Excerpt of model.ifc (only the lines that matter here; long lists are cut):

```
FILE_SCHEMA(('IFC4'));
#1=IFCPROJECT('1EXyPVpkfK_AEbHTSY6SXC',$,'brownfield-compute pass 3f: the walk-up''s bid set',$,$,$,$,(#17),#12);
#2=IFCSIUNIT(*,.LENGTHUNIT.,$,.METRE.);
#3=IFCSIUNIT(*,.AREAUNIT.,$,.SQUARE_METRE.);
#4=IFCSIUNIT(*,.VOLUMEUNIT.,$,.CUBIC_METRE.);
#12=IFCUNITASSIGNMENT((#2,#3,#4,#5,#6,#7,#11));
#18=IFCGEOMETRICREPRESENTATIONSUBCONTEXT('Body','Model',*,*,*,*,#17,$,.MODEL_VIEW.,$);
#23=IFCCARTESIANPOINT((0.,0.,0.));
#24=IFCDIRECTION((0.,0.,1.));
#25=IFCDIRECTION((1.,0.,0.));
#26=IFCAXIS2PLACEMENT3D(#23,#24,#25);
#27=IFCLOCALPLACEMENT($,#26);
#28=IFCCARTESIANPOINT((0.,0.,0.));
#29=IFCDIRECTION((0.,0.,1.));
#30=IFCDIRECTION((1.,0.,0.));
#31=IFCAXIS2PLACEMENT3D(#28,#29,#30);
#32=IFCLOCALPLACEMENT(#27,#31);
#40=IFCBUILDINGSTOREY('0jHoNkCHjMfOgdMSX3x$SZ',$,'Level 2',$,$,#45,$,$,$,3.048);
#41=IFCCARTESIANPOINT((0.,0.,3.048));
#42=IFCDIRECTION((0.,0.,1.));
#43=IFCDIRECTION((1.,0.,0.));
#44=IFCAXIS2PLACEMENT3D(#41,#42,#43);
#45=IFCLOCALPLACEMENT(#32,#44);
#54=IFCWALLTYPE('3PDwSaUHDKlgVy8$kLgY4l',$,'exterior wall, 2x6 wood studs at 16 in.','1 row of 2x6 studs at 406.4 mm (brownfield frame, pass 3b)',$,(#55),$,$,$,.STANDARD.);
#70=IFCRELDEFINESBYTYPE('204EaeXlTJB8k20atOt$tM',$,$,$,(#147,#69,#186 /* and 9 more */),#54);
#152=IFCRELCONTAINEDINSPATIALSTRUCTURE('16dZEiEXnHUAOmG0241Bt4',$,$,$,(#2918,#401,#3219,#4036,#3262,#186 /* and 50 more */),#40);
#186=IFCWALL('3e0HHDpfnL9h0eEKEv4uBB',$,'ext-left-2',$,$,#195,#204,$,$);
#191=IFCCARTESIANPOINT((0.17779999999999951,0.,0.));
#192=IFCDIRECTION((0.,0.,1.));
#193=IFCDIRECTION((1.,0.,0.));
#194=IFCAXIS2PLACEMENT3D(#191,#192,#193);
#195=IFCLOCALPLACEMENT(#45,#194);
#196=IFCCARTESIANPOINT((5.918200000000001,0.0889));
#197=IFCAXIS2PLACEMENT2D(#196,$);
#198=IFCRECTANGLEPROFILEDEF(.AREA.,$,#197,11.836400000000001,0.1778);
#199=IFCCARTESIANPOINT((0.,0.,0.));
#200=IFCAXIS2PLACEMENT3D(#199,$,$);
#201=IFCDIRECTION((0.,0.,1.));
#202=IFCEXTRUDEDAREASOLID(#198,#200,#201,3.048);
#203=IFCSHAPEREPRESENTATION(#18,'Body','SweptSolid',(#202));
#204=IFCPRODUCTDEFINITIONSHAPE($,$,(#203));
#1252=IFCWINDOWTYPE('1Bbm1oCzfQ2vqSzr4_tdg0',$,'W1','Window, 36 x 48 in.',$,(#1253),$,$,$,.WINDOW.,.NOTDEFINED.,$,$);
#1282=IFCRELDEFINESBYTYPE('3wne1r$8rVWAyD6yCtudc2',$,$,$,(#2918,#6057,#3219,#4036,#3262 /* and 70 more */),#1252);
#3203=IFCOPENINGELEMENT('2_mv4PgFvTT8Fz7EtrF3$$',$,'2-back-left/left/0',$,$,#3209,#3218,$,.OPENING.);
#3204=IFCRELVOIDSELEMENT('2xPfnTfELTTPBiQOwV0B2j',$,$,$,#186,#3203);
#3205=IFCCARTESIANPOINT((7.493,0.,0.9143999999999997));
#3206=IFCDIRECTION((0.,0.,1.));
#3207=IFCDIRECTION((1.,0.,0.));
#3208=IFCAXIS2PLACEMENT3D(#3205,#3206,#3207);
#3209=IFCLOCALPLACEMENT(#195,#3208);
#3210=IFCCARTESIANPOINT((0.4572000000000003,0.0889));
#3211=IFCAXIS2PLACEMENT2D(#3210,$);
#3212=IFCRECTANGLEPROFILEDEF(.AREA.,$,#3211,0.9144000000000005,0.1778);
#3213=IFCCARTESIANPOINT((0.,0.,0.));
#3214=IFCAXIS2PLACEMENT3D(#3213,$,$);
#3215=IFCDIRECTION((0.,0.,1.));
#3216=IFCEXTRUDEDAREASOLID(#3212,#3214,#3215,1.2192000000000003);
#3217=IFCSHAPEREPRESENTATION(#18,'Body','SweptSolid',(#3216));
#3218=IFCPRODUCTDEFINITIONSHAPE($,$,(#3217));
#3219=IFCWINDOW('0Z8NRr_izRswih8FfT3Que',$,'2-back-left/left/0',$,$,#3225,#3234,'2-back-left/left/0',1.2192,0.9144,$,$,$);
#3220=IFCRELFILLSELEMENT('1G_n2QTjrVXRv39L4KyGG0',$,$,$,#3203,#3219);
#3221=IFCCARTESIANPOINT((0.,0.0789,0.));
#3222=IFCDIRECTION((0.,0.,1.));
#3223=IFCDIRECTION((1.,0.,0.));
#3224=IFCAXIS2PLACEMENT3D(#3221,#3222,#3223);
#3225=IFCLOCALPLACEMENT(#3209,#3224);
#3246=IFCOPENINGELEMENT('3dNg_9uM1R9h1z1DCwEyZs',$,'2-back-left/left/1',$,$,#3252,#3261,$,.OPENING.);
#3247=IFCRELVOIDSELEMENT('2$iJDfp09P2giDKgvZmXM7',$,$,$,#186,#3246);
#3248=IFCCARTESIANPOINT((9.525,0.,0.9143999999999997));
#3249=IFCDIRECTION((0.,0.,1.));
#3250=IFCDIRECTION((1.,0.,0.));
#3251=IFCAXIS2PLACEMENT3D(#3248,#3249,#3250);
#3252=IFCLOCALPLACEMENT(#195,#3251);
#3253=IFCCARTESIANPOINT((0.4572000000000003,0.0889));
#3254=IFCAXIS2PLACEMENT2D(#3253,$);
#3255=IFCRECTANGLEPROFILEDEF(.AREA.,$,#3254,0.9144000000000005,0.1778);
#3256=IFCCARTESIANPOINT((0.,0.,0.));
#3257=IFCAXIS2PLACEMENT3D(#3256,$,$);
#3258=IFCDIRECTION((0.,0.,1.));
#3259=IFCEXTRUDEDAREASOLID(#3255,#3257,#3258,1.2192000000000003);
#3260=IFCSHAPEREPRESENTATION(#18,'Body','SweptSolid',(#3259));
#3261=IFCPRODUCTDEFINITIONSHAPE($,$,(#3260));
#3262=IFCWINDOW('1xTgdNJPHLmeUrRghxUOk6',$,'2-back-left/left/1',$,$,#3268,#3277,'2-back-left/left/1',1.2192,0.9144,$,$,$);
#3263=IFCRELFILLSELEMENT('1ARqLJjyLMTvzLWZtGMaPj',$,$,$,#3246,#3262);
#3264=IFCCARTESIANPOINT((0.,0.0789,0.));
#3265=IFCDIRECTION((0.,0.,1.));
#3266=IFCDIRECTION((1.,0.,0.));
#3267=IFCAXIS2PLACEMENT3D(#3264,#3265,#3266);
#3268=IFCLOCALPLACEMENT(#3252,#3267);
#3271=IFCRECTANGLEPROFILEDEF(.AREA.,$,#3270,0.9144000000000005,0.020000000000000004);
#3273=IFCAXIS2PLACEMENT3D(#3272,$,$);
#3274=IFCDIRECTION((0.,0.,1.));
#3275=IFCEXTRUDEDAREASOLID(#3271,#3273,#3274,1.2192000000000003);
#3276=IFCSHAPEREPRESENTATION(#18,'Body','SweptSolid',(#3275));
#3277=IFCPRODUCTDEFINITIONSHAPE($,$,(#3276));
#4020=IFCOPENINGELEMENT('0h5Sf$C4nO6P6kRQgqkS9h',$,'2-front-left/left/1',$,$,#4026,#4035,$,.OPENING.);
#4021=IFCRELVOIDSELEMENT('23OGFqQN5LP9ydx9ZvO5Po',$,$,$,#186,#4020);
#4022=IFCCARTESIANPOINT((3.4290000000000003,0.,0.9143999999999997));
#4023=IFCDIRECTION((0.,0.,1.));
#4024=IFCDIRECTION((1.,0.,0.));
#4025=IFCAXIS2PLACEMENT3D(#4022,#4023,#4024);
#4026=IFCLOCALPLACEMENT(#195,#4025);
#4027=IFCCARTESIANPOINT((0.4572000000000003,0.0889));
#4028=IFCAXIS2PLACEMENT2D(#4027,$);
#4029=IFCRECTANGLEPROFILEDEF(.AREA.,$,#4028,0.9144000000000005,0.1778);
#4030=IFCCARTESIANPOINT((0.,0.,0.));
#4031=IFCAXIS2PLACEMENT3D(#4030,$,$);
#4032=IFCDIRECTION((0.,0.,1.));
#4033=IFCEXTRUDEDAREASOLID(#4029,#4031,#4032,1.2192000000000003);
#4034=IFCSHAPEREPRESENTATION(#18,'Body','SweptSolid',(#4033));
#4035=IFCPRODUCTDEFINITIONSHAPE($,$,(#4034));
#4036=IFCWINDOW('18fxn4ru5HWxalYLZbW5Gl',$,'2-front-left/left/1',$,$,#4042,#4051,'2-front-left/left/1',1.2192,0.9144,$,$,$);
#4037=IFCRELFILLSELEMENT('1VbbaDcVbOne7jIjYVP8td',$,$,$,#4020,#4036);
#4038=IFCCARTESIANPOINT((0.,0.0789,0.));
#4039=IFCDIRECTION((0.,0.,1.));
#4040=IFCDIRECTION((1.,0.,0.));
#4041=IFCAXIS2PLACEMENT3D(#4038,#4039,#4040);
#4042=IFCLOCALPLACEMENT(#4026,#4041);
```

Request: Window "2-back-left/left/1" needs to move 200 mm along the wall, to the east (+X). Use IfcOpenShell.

```python
import ifcopenshell
import ifcopenshell.api.geometry
import ifcopenshell.util.placement
import ifcopenshell.util.unit

model = ifcopenshell.open("model.ifc")
unit_scale = ifcopenshell.util.unit.calculate_unit_scale(model)

window = model.by_guid("1xTgdNJPHLmeUrRghxUOk6")
opening = window.FillsVoids[0].RelatingOpeningElement
wall = opening.VoidsElements[0].RelatingBuildingElement

wall_matrix = ifcopenshell.util.placement.get_local_placement(wall.ObjectPlacement)
shift = wall_matrix[:3, 0] * 0.2 / unit_scale
before = ifcopenshell.util.placement.get_local_placement(window.ObjectPlacement)[:3, 3].copy()

# The window is placed relative to its opening, so it follows when the opening moves.
matrix = ifcopenshell.util.placement.get_local_placement(opening.ObjectPlacement)
matrix[:3, 3] += shift
ifcopenshell.api.geometry.edit_object_placement(
    model, product=opening, matrix=matrix, is_si=False, should_transform_children=True
)

after = ifcopenshell.util.placement.get_local_placement(window.ObjectPlacement)[:3, 3]
print("window moved by", (after - before).round(3) + 0.0)

model.write("model-out.ifc")
```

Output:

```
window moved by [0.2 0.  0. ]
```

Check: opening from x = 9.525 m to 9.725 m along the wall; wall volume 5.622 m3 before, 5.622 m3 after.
